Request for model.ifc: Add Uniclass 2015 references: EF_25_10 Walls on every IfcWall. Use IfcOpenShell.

First a look at what the model holds.

```python
import ifcopenshell

model = ifcopenshell.open("model.ifc")
print(model.schema)
print("classifications:", [c.Name for c in model.by_type("IfcClassification")])
for ifc_class in ("IfcDoor", "IfcRoof", "IfcStair", "IfcWall", "IfcWindow"):
    print(ifc_class, len(model.by_type(ifc_class)))
```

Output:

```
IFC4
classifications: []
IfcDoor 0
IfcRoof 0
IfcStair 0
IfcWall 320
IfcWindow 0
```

```python
import ifcopenshell
import ifcopenshell.api.classification

model = ifcopenshell.open("model.ifc")

system = ifcopenshell.api.classification.add_classification(model, classification="Uniclass 2015")

codes = {
    "IfcWall": ("EF_25_10", "Walls"),
}
for ifc_class, (code, name) in codes.items():
    products = model.by_type(ifc_class)
    ifcopenshell.api.classification.add_reference(
        model, products=products, classification=system, identification=code, name=name
    )
    print(code, len(products))

model.write("model_updated.ifc")
```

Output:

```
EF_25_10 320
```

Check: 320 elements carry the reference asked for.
